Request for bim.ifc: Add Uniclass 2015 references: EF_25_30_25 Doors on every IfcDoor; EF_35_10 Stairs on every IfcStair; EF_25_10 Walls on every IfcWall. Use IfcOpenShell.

First a look at what the model holds.

```python
import ifcopenshell

model = ifcopenshell.open("bim.ifc")
print(model.schema)
print("classifications:", [c.Name for c in model.by_type("IfcClassification")])
for ifc_class in ("IfcDoor", "IfcRoof", "IfcStair", "IfcWall", "IfcWindow"):
    print(ifc_class, len(model.by_type(ifc_class)))
```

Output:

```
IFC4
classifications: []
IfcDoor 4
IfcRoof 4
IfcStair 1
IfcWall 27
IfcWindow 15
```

```python
import ifcopenshell
import ifcopenshell.api.classification

model = ifcopenshell.open("bim.ifc")

system = ifcopenshell.api.classification.add_classification(model, classification="Uniclass 2015")

codes = {
    "IfcDoor": ("EF_25_30_25", "Doors"),
    "IfcStair": ("EF_35_10", "Stairs"),
    "IfcWall": ("EF_25_10", "Walls"),
}
for ifc_class, (code, name) in codes.items():
    products = model.by_type(ifc_class)
    ifcopenshell.api.classification.add_reference(
        model, products=products, classification=system, identification=code, name=name
    )
    print(code, len(products))

model.write("bim_rev.ifc")
```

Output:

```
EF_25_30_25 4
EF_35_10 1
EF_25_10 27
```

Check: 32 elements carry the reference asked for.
